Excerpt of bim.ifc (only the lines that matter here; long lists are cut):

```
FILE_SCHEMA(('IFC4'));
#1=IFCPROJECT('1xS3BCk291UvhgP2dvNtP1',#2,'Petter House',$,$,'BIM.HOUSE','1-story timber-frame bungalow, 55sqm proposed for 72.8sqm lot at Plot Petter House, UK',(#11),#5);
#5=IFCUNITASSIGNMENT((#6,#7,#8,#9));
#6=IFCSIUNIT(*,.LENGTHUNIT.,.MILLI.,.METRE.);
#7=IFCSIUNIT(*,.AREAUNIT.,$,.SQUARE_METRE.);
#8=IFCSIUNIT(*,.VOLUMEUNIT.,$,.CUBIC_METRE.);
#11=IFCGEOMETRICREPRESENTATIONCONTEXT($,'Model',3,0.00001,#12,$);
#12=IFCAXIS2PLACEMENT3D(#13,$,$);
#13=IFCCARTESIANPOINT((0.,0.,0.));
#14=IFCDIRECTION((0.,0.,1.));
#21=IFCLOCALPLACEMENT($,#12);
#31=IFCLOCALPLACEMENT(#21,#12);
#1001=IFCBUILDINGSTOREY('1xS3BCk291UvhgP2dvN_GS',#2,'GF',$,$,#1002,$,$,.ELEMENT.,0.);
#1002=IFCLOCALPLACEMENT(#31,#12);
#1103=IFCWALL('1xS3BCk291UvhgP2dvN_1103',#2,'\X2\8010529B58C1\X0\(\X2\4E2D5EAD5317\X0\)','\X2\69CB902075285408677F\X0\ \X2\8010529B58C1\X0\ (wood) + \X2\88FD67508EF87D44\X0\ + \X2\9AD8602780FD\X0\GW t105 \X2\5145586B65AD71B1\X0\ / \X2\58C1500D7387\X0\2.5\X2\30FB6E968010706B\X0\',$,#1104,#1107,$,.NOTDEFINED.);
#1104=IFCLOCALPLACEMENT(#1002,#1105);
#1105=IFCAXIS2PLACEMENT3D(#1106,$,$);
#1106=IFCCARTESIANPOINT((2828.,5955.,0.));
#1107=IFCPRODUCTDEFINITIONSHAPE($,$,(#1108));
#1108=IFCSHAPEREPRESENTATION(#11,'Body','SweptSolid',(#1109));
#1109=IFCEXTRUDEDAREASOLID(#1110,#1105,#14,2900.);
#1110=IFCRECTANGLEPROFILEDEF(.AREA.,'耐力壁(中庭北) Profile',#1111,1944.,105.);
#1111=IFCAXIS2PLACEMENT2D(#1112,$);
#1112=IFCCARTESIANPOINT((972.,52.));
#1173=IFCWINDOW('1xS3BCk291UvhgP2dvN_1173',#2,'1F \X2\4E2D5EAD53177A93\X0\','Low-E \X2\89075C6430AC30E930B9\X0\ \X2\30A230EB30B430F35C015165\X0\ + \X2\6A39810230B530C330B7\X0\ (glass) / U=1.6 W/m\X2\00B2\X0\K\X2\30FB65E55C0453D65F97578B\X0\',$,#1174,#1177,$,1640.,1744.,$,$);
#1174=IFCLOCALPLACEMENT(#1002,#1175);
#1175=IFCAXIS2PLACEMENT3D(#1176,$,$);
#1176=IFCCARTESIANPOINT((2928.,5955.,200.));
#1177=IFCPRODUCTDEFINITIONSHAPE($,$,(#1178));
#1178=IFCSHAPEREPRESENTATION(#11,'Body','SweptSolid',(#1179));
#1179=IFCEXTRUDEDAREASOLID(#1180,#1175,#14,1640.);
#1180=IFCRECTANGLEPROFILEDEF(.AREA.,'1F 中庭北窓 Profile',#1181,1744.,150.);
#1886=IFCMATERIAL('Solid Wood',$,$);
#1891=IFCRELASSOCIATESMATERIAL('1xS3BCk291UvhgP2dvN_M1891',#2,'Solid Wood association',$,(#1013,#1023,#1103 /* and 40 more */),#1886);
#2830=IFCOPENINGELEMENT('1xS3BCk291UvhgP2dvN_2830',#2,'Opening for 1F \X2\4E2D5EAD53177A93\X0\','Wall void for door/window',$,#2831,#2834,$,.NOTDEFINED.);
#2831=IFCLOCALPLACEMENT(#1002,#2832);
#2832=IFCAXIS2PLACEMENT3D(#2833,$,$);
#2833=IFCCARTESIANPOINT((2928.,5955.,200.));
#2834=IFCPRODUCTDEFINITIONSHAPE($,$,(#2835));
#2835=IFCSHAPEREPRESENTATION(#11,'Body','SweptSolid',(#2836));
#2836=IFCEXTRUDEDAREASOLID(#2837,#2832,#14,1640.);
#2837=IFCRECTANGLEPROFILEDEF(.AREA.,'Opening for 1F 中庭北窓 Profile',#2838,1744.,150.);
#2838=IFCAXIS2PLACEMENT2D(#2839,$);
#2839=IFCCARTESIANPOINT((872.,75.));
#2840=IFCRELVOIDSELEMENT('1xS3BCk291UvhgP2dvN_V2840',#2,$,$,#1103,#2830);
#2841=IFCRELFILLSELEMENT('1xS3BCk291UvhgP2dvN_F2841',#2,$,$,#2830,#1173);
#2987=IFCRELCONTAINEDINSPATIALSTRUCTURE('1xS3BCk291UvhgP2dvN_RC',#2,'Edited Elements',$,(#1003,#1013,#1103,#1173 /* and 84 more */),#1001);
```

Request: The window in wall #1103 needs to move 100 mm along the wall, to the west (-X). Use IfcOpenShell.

```python
import ifcopenshell
import ifcopenshell.api.geometry
import ifcopenshell.util.placement

model = ifcopenshell.open("bim.ifc")

window = model.by_guid("1xS3BCk291UvhgP2dvN_1173")
opening = window.FillsVoids[0].RelatingOpeningElement
wall = opening.VoidsElements[0].RelatingBuildingElement

wall_matrix = ifcopenshell.util.placement.get_local_placement(wall.ObjectPlacement)
shift = wall_matrix[:3, 0] * -100.0
before = ifcopenshell.util.placement.get_local_placement(window.ObjectPlacement)[:3, 3].copy()

# The window is not placed relative to its opening, so move both.
for product in (opening, window):
    matrix = ifcopenshell.util.placement.get_local_placement(product.ObjectPlacement)
    matrix[:3, 3] += shift
    ifcopenshell.api.geometry.edit_object_placement(model, product=product, matrix=matrix, is_si=False)

after = ifcopenshell.util.placement.get_local_placement(window.ObjectPlacement)[:3, 3]
print("window moved by", (after - before).round(3) + 0.0)

model.write("bim_rev.ifc")
```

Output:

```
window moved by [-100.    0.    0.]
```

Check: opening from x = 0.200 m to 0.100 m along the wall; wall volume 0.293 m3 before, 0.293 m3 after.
